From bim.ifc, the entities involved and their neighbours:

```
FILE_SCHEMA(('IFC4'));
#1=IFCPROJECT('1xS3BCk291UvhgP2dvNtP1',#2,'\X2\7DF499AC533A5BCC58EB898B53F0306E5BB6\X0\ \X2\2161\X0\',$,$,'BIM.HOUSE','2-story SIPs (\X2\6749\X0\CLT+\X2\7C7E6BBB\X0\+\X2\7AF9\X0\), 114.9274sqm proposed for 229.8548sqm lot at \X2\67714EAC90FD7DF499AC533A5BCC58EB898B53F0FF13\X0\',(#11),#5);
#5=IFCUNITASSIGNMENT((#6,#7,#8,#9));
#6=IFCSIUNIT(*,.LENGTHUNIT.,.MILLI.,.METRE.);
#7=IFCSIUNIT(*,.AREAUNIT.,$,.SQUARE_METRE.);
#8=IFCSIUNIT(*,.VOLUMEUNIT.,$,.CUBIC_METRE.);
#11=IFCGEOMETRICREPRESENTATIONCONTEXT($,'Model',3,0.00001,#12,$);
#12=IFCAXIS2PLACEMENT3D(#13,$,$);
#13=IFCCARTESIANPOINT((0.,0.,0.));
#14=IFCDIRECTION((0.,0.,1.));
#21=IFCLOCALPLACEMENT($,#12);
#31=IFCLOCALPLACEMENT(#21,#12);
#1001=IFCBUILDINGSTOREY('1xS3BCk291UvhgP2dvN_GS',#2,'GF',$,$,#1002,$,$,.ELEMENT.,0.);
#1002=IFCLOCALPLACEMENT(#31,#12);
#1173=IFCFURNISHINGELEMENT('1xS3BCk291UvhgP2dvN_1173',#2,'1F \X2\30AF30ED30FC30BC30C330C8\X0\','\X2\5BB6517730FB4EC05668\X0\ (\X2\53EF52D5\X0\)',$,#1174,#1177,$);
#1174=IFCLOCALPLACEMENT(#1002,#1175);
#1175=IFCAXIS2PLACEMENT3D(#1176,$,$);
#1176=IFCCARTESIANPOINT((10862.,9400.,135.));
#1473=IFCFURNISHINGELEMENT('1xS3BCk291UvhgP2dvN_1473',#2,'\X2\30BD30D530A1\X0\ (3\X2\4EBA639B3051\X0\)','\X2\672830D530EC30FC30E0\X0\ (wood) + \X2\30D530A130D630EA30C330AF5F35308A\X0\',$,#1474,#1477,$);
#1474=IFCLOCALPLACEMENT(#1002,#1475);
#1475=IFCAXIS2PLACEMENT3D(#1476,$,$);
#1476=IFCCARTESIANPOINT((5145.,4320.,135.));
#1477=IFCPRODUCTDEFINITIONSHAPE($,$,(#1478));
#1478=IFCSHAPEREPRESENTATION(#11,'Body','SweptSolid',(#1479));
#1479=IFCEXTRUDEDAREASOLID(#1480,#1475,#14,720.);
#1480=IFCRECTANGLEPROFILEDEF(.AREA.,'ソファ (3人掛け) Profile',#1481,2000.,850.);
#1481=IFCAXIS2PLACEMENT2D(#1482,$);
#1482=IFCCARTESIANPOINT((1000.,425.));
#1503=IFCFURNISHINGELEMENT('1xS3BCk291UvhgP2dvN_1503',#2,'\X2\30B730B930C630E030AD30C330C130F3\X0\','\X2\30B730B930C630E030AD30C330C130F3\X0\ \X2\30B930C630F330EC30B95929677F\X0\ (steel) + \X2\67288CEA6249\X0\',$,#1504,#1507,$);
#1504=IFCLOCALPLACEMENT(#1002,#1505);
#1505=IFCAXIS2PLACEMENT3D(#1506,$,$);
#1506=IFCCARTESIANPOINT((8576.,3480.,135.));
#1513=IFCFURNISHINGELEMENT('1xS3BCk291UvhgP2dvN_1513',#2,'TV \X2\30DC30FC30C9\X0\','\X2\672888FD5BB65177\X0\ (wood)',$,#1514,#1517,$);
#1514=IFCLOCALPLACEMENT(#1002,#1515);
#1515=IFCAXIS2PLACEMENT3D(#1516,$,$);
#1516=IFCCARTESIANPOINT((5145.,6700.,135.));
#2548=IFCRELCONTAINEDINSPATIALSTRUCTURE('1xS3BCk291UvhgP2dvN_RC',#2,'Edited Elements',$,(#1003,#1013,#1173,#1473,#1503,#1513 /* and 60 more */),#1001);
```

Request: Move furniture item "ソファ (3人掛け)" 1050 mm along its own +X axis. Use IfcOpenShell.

```python
import ifcopenshell
import ifcopenshell.api.geometry
import ifcopenshell.util.placement
import ifcopenshell.util.unit

model = ifcopenshell.open("bim.ifc")
unit_scale = ifcopenshell.util.unit.calculate_unit_scale(model)

item = model.by_guid("1xS3BCk291UvhgP2dvN_1473")
matrix = ifcopenshell.util.placement.get_local_placement(item.ObjectPlacement)
matrix[:3, 3] += matrix[:3, 0] * 1.05 / unit_scale
ifcopenshell.api.geometry.edit_object_placement(model, product=item, matrix=matrix, is_si=False)

print(ifcopenshell.util.placement.get_local_placement(item.ObjectPlacement).round(3) + 0.0)

model.write("bim_v2.ifc")
```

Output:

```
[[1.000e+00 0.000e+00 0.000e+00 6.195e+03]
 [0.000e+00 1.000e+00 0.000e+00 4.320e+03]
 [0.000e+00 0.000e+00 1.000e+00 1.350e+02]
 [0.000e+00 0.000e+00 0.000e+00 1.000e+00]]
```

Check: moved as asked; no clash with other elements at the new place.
